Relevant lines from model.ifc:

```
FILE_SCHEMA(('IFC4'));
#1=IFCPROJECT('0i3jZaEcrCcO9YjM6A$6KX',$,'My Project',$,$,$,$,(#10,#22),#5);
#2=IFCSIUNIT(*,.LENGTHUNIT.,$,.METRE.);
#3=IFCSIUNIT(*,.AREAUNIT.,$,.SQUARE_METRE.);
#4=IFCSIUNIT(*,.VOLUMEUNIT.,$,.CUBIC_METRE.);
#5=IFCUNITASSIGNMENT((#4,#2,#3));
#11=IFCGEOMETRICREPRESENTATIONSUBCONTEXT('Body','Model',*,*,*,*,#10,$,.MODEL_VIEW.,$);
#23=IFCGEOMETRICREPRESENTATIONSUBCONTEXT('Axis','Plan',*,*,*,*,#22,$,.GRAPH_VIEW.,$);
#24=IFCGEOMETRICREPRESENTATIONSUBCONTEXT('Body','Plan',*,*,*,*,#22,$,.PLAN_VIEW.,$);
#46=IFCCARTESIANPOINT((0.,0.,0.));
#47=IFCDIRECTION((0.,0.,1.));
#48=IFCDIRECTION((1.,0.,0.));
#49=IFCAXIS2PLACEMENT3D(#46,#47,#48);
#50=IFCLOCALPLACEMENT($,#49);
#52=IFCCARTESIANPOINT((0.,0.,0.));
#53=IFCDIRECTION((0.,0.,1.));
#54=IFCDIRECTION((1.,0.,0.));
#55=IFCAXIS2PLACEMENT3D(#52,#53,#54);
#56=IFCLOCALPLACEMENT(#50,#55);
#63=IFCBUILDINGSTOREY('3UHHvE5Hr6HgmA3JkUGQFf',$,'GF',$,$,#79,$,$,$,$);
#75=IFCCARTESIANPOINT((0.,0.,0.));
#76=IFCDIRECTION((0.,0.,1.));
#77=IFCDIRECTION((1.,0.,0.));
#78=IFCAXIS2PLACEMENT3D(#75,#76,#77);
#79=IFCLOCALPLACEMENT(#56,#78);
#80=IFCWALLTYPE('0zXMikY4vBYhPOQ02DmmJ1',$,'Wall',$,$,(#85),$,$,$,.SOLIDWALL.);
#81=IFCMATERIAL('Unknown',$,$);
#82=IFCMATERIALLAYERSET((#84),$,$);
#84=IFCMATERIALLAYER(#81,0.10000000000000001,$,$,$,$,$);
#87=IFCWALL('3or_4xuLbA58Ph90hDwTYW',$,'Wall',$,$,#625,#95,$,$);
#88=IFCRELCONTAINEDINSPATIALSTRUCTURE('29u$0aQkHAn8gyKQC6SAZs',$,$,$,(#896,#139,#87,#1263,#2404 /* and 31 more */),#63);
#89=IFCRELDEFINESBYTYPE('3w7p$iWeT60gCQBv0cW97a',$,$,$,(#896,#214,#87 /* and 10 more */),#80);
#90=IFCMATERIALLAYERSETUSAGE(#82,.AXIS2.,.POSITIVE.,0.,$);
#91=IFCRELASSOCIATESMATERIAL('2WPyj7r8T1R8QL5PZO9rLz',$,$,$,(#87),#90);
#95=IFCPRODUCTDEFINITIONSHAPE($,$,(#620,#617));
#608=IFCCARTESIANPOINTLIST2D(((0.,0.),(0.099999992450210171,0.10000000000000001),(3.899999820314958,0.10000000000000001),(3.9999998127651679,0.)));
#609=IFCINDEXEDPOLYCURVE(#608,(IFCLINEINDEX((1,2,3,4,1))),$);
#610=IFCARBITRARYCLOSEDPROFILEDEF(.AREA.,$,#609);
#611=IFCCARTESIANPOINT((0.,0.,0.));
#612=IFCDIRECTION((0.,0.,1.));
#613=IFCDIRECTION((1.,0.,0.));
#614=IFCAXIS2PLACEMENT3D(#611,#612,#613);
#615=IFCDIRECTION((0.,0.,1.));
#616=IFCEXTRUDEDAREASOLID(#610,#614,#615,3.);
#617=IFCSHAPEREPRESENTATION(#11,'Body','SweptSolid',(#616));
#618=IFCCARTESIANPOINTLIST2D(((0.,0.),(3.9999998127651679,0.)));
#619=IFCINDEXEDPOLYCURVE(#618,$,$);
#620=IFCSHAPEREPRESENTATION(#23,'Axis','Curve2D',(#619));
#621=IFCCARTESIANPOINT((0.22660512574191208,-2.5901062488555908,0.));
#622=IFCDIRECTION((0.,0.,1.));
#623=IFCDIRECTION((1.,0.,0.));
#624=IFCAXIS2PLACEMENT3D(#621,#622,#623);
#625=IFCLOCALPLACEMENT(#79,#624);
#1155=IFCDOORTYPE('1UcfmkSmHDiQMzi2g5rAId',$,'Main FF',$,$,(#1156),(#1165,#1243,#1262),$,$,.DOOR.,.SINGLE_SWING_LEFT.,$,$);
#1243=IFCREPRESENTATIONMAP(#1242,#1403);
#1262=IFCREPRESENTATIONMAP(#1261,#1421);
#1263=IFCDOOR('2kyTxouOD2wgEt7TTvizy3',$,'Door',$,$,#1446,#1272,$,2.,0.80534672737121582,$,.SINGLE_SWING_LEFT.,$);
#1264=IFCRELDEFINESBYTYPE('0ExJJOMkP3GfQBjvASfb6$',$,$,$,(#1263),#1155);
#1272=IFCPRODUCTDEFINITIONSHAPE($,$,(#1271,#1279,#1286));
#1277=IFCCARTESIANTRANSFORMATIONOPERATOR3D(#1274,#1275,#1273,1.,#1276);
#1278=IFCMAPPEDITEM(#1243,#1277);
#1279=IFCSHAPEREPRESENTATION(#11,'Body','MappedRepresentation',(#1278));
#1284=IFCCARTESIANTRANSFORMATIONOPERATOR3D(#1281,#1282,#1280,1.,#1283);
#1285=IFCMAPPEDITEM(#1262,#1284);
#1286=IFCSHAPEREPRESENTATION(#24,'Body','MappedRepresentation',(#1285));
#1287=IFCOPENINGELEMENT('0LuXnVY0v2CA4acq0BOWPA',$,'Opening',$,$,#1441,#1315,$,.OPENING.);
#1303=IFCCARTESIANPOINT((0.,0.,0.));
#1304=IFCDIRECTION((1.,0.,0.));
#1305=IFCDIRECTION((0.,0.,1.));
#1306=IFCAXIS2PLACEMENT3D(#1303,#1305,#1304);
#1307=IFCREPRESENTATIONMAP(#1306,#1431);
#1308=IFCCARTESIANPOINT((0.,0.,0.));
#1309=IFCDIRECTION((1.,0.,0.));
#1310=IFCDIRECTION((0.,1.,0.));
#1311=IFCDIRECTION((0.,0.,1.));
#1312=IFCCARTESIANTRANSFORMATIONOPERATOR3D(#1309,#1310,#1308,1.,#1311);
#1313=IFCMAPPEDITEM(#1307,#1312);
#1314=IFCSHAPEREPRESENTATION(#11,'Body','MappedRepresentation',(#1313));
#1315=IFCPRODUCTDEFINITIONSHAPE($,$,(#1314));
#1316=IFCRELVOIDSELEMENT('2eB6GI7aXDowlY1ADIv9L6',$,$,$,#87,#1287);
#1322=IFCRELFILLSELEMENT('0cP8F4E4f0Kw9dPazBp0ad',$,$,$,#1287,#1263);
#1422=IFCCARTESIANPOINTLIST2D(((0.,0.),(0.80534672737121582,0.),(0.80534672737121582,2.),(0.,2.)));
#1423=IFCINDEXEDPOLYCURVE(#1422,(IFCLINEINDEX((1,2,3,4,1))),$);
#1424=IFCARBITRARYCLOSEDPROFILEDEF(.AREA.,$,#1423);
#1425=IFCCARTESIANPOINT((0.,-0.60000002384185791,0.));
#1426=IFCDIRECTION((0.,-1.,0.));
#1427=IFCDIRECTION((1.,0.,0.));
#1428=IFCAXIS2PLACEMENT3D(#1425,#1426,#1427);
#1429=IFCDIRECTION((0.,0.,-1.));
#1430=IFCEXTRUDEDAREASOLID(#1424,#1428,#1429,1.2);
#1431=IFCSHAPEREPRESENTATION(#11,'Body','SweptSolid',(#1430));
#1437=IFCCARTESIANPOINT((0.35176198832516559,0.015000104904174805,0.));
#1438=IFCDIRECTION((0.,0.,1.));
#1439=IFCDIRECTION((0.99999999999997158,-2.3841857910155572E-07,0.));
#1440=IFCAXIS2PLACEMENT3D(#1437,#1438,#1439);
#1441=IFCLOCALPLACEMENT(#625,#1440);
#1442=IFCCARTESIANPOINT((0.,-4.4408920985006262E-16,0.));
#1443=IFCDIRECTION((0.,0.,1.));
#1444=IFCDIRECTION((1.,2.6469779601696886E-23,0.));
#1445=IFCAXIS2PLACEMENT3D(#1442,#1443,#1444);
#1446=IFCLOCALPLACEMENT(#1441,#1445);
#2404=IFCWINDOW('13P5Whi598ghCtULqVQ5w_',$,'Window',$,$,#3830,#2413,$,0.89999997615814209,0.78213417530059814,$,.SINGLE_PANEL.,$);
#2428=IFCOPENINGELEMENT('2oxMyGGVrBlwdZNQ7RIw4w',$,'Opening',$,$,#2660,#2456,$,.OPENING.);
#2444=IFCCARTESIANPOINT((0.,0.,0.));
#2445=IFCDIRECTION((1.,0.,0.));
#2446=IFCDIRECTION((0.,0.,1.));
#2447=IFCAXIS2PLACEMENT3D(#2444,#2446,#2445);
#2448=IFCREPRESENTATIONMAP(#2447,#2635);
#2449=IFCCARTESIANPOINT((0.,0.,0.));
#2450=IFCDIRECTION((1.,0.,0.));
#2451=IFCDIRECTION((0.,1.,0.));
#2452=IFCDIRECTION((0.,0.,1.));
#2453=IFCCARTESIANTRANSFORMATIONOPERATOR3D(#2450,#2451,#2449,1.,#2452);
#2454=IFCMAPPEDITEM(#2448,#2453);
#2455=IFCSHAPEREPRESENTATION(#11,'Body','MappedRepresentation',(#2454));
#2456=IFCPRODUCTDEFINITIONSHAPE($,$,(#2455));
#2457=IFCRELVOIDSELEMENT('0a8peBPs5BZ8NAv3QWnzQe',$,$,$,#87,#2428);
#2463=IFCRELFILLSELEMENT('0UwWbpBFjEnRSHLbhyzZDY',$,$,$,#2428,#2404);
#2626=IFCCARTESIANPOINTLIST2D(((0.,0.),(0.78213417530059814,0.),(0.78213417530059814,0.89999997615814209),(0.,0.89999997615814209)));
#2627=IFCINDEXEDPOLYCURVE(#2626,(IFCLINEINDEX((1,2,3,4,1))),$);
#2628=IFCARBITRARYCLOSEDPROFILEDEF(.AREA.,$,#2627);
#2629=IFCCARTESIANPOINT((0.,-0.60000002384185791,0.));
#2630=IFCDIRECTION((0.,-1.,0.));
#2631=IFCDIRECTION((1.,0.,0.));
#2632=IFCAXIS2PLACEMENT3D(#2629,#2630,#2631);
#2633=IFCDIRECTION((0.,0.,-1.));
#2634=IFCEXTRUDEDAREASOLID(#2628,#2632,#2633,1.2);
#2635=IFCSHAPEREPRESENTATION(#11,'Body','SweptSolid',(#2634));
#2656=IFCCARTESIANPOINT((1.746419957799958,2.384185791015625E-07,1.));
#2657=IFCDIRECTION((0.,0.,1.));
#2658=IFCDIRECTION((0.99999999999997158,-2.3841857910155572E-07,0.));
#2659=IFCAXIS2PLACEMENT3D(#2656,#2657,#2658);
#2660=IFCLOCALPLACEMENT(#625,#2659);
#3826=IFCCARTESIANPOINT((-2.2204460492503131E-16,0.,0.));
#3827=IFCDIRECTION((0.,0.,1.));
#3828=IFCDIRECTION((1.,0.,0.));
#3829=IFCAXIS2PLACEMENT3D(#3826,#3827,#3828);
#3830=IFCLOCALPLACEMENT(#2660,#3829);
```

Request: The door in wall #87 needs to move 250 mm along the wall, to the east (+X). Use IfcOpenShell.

```python
import ifcopenshell
import ifcopenshell.api.geometry
import ifcopenshell.util.placement
import ifcopenshell.util.unit

model = ifcopenshell.open("model.ifc")
unit_scale = ifcopenshell.util.unit.calculate_unit_scale(model)

door = model.by_id(1263)
opening = door.FillsVoids[0].RelatingOpeningElement
wall = opening.VoidsElements[0].RelatingBuildingElement

wall_matrix = ifcopenshell.util.placement.get_local_placement(wall.ObjectPlacement)
shift = wall_matrix[:3, 0] * 0.25 / unit_scale
before = ifcopenshell.util.placement.get_local_placement(door.ObjectPlacement)[:3, 3].copy()

# The door is placed relative to its opening, so it follows when the opening moves.
matrix = ifcopenshell.util.placement.get_local_placement(opening.ObjectPlacement)
matrix[:3, 3] += shift
ifcopenshell.api.geometry.edit_object_placement(
    model, product=opening, matrix=matrix, is_si=False, should_transform_children=True
)

after = ifcopenshell.util.placement.get_local_placement(door.ObjectPlacement)[:3, 3]
print("door moved by", (after - before).round(3) + 0.0)

model.write("model-out.ifc")
```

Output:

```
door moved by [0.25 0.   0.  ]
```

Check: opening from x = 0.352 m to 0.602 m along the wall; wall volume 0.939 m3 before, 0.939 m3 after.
